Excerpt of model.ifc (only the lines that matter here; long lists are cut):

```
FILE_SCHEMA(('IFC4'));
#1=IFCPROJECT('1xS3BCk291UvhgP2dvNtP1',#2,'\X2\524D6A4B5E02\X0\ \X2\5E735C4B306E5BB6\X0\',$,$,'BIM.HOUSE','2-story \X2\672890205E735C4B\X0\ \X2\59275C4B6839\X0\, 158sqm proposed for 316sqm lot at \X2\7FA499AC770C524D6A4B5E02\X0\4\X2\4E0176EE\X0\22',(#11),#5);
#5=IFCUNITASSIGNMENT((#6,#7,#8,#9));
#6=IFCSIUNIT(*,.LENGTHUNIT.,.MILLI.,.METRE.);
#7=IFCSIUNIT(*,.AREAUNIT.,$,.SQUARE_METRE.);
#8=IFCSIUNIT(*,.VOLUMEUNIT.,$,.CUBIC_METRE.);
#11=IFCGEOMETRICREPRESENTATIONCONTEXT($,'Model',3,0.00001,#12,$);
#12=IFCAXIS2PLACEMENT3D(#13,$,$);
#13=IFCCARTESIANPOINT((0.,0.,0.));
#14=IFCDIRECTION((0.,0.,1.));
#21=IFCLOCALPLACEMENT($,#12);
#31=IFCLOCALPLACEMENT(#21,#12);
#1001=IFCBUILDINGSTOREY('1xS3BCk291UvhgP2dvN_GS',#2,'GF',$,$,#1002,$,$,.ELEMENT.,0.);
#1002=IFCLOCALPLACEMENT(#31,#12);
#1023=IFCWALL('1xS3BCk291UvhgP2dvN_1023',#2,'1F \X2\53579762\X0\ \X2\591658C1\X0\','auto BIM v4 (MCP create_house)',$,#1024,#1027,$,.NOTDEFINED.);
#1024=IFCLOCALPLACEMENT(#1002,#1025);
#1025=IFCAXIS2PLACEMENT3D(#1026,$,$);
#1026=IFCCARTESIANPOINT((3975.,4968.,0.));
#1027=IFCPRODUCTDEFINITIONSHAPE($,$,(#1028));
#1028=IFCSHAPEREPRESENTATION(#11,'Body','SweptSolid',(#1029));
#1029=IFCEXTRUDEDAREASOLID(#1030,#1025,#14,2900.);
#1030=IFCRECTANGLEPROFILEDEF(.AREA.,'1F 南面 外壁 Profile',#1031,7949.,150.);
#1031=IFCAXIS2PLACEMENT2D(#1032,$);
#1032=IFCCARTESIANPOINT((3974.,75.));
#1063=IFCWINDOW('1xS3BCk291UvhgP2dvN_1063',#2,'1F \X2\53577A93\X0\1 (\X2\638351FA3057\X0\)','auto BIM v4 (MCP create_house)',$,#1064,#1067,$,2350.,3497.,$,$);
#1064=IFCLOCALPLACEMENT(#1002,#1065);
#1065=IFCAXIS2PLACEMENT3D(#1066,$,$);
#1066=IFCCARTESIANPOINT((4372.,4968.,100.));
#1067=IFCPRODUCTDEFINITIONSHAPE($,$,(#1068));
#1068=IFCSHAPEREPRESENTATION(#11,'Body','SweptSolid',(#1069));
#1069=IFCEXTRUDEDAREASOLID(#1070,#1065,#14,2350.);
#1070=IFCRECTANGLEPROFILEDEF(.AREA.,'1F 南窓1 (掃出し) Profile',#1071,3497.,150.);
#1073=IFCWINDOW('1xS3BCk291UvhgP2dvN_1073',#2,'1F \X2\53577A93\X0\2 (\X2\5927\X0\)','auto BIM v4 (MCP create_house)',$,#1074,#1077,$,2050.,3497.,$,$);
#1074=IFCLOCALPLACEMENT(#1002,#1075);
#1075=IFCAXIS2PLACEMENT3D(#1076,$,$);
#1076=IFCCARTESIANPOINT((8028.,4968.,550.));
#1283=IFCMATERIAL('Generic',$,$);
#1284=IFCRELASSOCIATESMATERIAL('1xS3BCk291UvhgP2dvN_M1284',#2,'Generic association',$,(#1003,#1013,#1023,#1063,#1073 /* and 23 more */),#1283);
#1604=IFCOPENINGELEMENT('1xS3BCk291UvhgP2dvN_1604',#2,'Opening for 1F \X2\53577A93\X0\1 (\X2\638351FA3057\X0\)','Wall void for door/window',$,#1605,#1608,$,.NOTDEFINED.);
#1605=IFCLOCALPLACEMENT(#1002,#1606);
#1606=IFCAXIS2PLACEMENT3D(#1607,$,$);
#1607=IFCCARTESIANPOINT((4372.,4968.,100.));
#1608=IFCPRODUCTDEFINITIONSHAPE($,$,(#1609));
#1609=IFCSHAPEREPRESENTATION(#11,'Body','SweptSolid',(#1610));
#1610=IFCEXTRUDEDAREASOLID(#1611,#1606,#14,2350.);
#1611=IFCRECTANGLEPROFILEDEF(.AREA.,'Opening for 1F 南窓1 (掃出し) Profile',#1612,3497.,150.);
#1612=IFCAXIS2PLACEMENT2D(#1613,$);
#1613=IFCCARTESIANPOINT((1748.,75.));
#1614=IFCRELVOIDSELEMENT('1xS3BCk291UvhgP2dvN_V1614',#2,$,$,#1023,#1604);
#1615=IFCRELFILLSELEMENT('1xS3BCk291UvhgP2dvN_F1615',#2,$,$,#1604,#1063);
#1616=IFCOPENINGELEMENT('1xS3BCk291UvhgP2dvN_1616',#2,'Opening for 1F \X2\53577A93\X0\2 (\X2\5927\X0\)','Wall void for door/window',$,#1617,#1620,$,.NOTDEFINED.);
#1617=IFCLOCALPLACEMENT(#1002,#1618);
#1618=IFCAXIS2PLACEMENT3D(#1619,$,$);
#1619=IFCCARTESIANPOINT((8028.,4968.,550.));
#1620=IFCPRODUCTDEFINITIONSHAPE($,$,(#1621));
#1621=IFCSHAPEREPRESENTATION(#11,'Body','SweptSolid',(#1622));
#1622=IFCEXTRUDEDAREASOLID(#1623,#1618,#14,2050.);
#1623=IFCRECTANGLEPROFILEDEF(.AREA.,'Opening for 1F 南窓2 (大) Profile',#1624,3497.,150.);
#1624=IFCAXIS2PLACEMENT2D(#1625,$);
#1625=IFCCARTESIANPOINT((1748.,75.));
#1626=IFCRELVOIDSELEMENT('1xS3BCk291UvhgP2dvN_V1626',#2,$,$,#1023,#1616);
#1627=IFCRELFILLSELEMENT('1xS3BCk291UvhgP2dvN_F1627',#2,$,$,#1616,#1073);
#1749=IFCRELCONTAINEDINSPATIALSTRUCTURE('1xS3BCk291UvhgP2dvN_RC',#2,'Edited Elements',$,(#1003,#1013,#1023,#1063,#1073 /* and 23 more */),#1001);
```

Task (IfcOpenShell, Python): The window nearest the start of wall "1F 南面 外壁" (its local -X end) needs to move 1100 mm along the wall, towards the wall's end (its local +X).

```python
import ifcopenshell
import ifcopenshell.api.geometry
import ifcopenshell.util.placement

model = ifcopenshell.open("model.ifc")

window = model.by_guid("1xS3BCk291UvhgP2dvN_1063")
opening = window.FillsVoids[0].RelatingOpeningElement
wall = opening.VoidsElements[0].RelatingBuildingElement

wall_matrix = ifcopenshell.util.placement.get_local_placement(wall.ObjectPlacement)
shift = wall_matrix[:3, 0] * 1100.0
before = ifcopenshell.util.placement.get_local_placement(window.ObjectPlacement)[:3, 3].copy()

# The window is not placed relative to its opening, so move both.
for product in (opening, window):
    matrix = ifcopenshell.util.placement.get_local_placement(product.ObjectPlacement)
    matrix[:3, 3] += shift
    ifcopenshell.api.geometry.edit_object_placement(model, product=product, matrix=matrix, is_si=False)

after = ifcopenshell.util.placement.get_local_placement(window.ObjectPlacement)[:3, 3]
print("window moved by", (after - before).round(3) + 0.0)

model.write("model_updated.ifc")
```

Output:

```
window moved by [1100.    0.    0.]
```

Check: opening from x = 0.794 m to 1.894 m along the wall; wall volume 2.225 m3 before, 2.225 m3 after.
